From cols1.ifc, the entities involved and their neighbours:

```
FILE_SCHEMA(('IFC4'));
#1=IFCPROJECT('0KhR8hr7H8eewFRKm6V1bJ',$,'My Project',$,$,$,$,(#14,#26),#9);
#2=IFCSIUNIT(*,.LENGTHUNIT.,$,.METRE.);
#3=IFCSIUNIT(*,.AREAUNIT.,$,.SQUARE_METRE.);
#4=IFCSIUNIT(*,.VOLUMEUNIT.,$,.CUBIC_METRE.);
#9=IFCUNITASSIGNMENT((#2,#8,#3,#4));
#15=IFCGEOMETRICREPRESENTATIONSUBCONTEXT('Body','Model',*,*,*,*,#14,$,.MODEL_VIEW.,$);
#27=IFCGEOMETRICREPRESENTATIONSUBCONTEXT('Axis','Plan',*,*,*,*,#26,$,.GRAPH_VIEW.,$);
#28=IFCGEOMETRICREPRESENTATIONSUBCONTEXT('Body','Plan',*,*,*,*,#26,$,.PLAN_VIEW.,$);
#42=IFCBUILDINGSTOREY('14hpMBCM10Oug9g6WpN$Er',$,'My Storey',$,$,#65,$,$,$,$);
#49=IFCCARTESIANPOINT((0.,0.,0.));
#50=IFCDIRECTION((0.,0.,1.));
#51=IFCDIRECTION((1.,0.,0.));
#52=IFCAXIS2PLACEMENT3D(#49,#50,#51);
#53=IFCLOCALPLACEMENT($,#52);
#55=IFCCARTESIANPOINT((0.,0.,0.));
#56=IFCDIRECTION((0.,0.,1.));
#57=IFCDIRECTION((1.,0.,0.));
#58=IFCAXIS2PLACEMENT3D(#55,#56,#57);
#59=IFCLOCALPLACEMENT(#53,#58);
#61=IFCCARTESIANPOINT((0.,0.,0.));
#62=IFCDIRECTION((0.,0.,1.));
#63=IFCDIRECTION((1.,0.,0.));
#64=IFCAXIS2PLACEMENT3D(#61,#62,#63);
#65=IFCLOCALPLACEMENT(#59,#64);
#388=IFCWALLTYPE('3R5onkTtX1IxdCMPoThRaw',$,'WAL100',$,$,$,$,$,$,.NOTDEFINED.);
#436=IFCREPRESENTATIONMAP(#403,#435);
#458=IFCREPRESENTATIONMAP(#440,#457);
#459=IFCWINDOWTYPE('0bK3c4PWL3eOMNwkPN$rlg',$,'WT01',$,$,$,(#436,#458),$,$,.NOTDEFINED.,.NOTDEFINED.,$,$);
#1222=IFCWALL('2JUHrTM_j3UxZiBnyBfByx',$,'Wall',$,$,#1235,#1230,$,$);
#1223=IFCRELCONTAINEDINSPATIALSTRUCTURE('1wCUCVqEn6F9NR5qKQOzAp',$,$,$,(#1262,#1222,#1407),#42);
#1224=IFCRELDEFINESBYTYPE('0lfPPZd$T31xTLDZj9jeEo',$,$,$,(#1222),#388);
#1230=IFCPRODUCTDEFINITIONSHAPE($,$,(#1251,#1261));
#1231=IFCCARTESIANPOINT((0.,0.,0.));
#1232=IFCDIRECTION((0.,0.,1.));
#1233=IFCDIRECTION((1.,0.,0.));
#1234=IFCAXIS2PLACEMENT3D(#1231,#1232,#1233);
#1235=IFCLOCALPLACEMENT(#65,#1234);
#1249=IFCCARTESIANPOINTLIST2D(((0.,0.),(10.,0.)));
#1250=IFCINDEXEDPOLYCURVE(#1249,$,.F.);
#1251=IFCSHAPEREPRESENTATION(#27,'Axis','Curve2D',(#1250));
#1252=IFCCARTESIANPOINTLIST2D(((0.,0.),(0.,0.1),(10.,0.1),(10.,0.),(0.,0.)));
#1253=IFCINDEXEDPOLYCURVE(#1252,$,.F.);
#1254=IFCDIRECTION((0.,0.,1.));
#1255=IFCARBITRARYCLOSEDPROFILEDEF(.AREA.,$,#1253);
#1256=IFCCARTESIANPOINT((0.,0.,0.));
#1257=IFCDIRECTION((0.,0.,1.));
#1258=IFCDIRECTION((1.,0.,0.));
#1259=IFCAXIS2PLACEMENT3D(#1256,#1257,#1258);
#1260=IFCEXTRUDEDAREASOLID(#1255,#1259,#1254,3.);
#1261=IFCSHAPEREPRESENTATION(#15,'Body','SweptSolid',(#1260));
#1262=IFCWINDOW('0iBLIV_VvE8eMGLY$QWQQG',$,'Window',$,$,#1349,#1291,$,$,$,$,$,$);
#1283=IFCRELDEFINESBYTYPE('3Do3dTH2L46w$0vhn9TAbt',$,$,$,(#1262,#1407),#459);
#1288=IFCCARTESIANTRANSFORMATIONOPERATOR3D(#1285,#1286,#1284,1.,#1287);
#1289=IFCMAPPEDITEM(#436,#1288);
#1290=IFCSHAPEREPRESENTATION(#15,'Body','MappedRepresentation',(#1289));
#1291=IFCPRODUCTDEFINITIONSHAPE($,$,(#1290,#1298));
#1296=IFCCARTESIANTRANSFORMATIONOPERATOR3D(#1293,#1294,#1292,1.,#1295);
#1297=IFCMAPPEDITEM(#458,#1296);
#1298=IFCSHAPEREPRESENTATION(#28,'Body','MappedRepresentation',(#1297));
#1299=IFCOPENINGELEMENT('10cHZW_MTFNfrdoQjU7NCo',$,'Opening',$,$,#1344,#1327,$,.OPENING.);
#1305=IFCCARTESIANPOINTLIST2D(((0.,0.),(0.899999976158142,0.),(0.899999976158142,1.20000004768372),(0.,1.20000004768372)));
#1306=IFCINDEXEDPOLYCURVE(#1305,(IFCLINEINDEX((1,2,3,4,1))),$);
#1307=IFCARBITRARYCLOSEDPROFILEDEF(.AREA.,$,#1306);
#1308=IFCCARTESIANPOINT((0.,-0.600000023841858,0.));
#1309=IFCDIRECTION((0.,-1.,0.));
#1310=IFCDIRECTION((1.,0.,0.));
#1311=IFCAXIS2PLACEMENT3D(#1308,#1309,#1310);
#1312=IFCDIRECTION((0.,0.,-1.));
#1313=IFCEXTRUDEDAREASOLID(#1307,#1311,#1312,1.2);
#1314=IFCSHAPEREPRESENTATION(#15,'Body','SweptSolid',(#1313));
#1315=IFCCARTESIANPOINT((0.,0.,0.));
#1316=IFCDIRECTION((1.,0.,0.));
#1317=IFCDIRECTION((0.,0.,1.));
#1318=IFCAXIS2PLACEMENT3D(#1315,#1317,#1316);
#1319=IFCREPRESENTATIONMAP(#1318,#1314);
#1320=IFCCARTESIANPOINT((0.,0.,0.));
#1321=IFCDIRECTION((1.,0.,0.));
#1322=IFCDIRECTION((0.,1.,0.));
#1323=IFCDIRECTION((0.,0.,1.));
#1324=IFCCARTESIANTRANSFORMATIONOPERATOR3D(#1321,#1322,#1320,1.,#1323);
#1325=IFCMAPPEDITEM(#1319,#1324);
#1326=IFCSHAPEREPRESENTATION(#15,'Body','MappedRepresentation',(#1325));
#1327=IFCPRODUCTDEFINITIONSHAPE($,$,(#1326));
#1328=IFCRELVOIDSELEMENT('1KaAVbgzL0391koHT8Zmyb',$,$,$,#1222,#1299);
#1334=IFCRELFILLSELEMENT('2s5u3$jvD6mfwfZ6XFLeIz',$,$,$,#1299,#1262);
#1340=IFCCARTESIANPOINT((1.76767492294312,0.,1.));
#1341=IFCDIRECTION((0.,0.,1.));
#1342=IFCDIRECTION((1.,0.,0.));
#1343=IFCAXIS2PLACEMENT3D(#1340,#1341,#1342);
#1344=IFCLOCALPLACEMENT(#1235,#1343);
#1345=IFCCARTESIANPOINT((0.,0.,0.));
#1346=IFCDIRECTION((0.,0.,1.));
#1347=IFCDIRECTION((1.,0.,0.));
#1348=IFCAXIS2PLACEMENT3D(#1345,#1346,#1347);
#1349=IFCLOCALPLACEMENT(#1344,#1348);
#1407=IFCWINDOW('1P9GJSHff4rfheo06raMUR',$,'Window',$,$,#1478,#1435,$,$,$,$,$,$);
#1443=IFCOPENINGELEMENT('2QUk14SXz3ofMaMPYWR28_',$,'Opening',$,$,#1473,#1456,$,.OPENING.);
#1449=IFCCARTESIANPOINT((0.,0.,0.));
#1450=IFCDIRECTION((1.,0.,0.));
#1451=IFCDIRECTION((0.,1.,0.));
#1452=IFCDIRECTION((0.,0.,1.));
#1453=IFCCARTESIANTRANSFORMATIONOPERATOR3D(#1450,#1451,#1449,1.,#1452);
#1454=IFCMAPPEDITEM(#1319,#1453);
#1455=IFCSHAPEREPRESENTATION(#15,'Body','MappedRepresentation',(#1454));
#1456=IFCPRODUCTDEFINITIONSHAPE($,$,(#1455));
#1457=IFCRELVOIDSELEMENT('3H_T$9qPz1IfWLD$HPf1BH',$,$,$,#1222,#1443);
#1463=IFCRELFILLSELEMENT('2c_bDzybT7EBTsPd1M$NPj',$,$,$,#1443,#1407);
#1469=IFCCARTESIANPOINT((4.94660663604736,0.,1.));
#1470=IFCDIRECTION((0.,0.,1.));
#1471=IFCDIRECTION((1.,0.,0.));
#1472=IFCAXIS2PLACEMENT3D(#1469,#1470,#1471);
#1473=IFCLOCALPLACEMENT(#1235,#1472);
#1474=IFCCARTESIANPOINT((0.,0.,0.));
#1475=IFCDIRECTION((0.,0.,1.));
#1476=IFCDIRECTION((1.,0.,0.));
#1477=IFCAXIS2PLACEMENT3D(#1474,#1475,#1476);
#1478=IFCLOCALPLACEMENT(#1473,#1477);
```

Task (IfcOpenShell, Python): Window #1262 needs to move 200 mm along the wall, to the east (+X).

```python
import ifcopenshell
import ifcopenshell.api.geometry
import ifcopenshell.util.placement

model = ifcopenshell.open("cols1.ifc")

window = model.by_id(1262)
opening = window.FillsVoids[0].RelatingOpeningElement
wall = opening.VoidsElements[0].RelatingBuildingElement

wall_matrix = ifcopenshell.util.placement.get_local_placement(wall.ObjectPlacement)
shift = wall_matrix[:3, 0] * 0.2
before = ifcopenshell.util.placement.get_local_placement(window.ObjectPlacement)[:3, 3].copy()

# The window is placed relative to its opening, so it follows when the opening moves.
matrix = ifcopenshell.util.placement.get_local_placement(opening.ObjectPlacement)
matrix[:3, 3] += shift
ifcopenshell.api.geometry.edit_object_placement(
    model, product=opening, matrix=matrix, is_si=False, should_transform_children=True
)

after = ifcopenshell.util.placement.get_local_placement(window.ObjectPlacement)[:3, 3]
print("window moved by", (after - before).round(3) + 0.0)

model.write("cols1_v2.ifc")
```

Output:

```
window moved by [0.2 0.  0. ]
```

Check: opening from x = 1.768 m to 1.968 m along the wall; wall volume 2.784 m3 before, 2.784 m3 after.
